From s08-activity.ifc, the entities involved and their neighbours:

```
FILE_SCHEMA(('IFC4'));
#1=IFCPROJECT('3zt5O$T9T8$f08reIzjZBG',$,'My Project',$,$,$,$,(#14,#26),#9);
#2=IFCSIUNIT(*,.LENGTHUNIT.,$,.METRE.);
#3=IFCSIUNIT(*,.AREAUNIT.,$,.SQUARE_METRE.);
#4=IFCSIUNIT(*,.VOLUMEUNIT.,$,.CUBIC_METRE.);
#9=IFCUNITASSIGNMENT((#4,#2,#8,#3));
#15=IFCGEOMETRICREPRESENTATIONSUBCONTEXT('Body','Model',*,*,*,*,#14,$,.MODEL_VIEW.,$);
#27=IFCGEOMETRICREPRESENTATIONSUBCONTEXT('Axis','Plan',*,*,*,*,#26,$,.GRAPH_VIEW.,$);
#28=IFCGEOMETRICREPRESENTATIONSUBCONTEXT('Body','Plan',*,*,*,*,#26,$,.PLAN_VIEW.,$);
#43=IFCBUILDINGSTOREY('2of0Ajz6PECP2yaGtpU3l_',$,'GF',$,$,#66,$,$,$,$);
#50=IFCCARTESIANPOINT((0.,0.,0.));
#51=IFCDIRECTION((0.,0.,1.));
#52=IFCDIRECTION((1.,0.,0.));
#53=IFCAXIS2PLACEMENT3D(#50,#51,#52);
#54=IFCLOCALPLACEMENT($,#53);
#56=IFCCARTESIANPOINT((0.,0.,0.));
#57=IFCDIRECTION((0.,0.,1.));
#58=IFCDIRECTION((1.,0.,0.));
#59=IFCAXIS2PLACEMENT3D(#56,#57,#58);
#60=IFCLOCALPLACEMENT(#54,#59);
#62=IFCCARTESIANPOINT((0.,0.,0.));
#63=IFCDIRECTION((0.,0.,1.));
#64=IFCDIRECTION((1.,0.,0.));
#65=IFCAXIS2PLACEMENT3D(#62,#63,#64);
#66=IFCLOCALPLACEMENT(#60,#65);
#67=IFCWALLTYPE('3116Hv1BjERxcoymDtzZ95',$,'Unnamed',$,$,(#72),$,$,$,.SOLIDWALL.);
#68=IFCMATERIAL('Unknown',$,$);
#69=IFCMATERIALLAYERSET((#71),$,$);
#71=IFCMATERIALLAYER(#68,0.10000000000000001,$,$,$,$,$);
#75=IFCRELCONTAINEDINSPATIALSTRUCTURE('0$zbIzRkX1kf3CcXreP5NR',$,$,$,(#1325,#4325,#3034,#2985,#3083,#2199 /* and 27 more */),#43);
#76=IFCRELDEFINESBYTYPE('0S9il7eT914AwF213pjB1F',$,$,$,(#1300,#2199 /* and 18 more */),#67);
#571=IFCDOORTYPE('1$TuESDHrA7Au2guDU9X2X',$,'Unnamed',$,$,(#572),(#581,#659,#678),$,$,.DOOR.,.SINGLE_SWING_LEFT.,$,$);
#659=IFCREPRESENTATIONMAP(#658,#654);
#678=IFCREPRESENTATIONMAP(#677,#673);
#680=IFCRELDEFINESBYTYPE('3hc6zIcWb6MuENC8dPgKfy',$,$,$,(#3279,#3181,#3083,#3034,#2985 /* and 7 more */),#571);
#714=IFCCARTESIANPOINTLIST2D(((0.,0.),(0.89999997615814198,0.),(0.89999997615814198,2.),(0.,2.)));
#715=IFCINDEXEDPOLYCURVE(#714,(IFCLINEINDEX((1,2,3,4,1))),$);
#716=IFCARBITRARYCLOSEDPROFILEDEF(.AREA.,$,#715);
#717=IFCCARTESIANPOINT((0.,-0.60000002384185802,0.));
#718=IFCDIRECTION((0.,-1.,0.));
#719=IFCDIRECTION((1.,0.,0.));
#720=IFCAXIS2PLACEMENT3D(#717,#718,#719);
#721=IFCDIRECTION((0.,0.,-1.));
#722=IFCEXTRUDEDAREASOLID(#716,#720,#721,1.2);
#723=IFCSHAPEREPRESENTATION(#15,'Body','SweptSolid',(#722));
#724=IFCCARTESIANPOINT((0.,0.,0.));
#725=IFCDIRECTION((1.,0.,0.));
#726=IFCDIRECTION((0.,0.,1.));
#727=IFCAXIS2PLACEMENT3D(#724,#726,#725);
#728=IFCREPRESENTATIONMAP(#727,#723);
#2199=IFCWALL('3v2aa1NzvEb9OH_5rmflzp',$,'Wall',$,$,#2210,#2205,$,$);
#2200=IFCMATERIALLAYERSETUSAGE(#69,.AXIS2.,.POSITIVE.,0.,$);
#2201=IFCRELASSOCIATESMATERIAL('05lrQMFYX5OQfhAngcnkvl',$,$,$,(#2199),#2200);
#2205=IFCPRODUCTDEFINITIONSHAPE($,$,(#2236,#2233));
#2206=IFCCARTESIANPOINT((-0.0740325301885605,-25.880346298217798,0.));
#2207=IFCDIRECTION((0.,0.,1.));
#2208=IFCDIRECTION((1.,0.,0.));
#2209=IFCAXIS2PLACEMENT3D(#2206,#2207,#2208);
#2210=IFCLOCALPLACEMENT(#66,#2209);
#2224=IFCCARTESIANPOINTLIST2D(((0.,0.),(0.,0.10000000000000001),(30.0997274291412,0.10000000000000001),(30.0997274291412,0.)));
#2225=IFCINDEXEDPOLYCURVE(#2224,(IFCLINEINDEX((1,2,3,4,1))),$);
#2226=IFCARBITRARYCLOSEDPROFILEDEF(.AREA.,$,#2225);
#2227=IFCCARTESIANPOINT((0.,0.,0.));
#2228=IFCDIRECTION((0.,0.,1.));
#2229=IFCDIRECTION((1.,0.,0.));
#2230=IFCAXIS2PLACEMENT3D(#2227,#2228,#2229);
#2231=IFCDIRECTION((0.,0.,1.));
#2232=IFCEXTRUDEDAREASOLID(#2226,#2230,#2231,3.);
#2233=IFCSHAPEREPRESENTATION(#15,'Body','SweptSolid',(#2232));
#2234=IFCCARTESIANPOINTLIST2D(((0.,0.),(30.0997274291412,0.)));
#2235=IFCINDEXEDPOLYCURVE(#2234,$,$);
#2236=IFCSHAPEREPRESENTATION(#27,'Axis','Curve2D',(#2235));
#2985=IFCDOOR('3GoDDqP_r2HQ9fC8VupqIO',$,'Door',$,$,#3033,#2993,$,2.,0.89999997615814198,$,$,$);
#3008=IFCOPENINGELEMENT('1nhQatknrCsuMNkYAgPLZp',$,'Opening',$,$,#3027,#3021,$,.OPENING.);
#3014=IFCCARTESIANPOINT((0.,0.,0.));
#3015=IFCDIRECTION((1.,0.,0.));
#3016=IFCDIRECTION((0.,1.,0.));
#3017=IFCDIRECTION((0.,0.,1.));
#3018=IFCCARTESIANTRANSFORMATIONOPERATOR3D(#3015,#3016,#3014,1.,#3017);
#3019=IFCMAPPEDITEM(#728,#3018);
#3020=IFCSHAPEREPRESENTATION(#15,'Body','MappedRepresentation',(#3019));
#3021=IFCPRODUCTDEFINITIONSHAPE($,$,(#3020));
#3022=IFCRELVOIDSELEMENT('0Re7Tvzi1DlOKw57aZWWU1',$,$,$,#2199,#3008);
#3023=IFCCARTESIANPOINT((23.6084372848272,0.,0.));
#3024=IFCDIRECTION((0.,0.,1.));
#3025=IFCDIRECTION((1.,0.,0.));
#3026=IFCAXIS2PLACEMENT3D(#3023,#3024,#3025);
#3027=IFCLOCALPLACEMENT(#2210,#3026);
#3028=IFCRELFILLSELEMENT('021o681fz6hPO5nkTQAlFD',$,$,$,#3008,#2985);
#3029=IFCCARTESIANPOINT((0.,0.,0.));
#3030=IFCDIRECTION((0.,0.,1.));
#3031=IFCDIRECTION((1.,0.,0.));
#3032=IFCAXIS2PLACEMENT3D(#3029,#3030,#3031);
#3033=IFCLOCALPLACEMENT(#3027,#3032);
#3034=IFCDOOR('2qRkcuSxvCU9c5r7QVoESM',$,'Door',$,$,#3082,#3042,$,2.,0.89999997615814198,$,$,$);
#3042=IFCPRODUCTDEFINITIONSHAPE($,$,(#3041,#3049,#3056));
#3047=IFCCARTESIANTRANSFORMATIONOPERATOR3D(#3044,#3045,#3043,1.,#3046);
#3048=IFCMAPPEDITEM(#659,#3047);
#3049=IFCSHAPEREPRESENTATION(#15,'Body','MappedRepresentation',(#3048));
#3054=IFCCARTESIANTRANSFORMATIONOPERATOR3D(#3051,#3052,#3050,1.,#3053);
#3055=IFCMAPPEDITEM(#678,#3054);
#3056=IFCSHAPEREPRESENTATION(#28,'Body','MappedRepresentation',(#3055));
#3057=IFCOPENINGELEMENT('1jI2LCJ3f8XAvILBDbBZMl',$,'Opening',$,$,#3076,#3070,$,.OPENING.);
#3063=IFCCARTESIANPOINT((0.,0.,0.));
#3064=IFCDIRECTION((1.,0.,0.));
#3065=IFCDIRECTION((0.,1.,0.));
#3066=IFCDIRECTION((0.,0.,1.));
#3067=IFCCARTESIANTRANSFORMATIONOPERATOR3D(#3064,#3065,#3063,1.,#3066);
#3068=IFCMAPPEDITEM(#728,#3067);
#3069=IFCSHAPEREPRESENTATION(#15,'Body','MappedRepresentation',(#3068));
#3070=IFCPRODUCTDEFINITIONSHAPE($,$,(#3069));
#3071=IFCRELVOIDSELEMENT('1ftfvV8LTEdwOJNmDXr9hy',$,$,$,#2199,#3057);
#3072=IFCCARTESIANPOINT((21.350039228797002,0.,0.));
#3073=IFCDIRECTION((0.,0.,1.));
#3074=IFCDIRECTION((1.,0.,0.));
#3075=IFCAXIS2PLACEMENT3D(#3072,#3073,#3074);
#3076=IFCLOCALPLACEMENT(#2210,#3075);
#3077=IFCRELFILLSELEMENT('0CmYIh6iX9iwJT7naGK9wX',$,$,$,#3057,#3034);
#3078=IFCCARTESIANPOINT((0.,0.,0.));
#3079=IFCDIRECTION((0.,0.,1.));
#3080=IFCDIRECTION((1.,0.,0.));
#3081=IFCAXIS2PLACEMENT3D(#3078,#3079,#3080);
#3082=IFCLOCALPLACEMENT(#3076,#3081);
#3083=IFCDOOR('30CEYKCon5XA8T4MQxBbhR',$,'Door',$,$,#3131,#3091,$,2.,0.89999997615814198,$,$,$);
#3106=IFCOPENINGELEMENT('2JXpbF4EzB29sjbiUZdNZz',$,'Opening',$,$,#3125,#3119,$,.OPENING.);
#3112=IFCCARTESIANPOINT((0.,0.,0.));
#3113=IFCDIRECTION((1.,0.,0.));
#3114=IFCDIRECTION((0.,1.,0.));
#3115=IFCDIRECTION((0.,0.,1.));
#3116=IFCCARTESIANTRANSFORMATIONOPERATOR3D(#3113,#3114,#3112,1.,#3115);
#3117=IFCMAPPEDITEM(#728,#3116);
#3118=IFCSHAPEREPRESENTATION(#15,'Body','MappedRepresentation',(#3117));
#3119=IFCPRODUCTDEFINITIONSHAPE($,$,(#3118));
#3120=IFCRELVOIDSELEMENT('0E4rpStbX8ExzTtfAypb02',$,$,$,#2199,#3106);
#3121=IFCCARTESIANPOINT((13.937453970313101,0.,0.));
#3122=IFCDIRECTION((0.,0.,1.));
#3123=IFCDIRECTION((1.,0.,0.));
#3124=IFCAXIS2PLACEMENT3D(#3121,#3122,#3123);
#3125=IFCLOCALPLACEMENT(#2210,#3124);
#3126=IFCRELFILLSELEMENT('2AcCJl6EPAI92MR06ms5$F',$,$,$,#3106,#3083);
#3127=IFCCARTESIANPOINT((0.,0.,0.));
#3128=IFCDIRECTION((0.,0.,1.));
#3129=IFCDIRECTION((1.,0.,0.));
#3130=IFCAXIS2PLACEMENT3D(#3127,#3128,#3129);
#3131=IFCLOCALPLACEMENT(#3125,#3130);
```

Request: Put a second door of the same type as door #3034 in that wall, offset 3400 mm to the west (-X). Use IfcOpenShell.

```python
import ifcopenshell
import ifcopenshell.api.feature
import ifcopenshell.api.geometry
import ifcopenshell.api.root
import ifcopenshell.geom
import ifcopenshell.util.element
import ifcopenshell.util.placement
import ifcopenshell.util.shape

model = ifcopenshell.open("s08-activity.ifc")
settings = ifcopenshell.geom.settings()


def volume(element):
    """Net volume in cubic metres, openings subtracted."""
    shape = ifcopenshell.geom.create_shape(settings, element)
    return ifcopenshell.util.shape.get_volume(shape.geometry)


door = model.by_id(3034)
opening = door.FillsVoids[0].RelatingOpeningElement
wall = opening.VoidsElements[0].RelatingBuildingElement
before = volume(wall)
shift = ifcopenshell.util.placement.get_local_placement(wall.ObjectPlacement)[:3, 0] * -3.4

# copy_class copies the void relationship, type, container and properties, but no geometry.
new_opening = ifcopenshell.api.root.copy_class(model, product=opening)
new_opening.Representation = ifcopenshell.util.element.copy_deep(
    model, opening.Representation, exclude=["IfcGeometricRepresentationContext", "IfcRepresentationMap"]
)
new_door = ifcopenshell.api.root.copy_class(model, product=door)
new_door.Representation = ifcopenshell.util.element.copy_deep(
    model, door.Representation, exclude=["IfcGeometricRepresentationContext", "IfcRepresentationMap"]
)
ifcopenshell.api.feature.add_filling(model, opening=new_opening, element=new_door)

for old, new in ((opening, new_opening), (door, new_door)):
    matrix = ifcopenshell.util.placement.get_local_placement(old.ObjectPlacement)
    matrix[:3, 3] += shift
    ifcopenshell.api.geometry.edit_object_placement(model, product=new, matrix=matrix, is_si=False)

after = volume(wall)

print(f"wall volume {before:.3f} -> {after:.3f} m3")

model.write("s08-activity_rev.ifc")
```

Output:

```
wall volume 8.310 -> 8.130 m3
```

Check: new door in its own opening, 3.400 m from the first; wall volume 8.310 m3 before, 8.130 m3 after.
